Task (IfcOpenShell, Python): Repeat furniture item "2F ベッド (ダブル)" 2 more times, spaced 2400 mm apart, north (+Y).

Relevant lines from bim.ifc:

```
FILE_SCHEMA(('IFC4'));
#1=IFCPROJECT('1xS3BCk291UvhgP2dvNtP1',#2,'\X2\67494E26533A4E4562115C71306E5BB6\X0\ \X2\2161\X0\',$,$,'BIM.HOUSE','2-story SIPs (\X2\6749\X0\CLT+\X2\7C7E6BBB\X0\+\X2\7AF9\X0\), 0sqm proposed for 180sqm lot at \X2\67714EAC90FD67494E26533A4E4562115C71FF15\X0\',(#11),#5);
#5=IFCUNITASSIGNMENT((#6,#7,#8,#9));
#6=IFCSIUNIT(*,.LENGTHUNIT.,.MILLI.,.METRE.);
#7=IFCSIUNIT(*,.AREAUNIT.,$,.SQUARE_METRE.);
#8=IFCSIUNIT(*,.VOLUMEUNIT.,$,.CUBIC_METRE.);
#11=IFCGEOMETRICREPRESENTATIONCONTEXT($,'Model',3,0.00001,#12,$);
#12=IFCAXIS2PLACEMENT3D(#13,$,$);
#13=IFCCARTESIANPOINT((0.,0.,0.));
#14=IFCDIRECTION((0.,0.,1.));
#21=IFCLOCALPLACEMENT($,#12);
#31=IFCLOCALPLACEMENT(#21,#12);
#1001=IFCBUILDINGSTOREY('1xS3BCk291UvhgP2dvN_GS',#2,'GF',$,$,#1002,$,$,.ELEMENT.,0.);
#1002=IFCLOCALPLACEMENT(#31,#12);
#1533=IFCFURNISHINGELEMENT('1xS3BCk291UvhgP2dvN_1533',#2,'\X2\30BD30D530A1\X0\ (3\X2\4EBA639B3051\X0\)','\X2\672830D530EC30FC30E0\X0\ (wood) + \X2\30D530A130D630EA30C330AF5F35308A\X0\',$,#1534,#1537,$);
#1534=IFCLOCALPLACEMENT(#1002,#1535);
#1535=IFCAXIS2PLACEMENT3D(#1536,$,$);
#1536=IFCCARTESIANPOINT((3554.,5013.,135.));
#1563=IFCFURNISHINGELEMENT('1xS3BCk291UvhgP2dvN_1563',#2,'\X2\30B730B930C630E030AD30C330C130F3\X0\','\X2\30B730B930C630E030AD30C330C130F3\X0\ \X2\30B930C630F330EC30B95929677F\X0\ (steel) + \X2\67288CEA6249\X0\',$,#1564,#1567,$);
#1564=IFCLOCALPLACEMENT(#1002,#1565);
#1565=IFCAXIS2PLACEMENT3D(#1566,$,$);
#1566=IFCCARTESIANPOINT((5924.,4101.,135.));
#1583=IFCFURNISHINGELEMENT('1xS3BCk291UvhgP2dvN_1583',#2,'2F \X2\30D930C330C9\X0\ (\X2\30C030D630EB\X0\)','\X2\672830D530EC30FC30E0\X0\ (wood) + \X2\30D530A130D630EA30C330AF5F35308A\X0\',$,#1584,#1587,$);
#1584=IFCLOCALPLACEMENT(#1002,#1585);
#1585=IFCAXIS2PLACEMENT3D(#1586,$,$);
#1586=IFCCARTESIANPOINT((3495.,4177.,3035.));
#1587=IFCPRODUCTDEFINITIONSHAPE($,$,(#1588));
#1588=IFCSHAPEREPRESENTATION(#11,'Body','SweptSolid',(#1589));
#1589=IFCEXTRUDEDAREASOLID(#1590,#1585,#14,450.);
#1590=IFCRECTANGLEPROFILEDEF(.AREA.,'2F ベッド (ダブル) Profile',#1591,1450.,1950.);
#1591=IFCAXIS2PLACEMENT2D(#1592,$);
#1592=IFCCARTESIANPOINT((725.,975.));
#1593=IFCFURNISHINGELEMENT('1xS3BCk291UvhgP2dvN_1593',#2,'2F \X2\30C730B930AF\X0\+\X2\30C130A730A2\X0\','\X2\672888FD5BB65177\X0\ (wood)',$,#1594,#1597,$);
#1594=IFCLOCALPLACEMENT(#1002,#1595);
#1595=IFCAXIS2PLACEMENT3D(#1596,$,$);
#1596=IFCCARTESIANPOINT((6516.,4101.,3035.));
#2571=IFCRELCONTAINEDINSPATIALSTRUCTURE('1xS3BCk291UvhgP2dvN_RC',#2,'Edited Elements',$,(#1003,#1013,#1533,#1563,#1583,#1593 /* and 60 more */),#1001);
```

```python
import numpy as np
import ifcopenshell
import ifcopenshell.api.geometry
import ifcopenshell.api.root
import ifcopenshell.util.element
import ifcopenshell.util.placement
import ifcopenshell.util.unit

model = ifcopenshell.open("bim.ifc")
unit_scale = ifcopenshell.util.unit.calculate_unit_scale(model)


def reuse_history(source, copy):
    """copy_class also copies each property set's owner history, people and application; keep the originals."""
    for rel in copy.IsDefinedBy:
        if rel.is_a("IfcRelDefinesByProperties") and (history := rel.RelatingPropertyDefinition.OwnerHistory):
            rel.RelatingPropertyDefinition.OwnerHistory = source.OwnerHistory
            ifcopenshell.util.element.remove_deep2(model, history)


source = model.by_guid("1xS3BCk291UvhgP2dvN_1583")
base = ifcopenshell.util.placement.get_local_placement(source.ObjectPlacement)
step = np.array([0.0, 1.0, 0.0]) * 2.4 / unit_scale

for i in range(1, 3):
    copy = ifcopenshell.api.root.copy_class(model, product=source)
    copy.Representation = ifcopenshell.util.element.copy_deep(
        model, source.Representation, exclude=["IfcGeometricRepresentationContext", "IfcRepresentationMap"]
    )
    reuse_history(source, copy)
    matrix = base.copy()
    matrix[:3, 3] += i * step
    print("added at", matrix[:3, 3].round(3) + 0.0)
    ifcopenshell.api.geometry.edit_object_placement(model, product=copy, matrix=matrix, is_si=False)

model.write("bim_rev.ifc")
```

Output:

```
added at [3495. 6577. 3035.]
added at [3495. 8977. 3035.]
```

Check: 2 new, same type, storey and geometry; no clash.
